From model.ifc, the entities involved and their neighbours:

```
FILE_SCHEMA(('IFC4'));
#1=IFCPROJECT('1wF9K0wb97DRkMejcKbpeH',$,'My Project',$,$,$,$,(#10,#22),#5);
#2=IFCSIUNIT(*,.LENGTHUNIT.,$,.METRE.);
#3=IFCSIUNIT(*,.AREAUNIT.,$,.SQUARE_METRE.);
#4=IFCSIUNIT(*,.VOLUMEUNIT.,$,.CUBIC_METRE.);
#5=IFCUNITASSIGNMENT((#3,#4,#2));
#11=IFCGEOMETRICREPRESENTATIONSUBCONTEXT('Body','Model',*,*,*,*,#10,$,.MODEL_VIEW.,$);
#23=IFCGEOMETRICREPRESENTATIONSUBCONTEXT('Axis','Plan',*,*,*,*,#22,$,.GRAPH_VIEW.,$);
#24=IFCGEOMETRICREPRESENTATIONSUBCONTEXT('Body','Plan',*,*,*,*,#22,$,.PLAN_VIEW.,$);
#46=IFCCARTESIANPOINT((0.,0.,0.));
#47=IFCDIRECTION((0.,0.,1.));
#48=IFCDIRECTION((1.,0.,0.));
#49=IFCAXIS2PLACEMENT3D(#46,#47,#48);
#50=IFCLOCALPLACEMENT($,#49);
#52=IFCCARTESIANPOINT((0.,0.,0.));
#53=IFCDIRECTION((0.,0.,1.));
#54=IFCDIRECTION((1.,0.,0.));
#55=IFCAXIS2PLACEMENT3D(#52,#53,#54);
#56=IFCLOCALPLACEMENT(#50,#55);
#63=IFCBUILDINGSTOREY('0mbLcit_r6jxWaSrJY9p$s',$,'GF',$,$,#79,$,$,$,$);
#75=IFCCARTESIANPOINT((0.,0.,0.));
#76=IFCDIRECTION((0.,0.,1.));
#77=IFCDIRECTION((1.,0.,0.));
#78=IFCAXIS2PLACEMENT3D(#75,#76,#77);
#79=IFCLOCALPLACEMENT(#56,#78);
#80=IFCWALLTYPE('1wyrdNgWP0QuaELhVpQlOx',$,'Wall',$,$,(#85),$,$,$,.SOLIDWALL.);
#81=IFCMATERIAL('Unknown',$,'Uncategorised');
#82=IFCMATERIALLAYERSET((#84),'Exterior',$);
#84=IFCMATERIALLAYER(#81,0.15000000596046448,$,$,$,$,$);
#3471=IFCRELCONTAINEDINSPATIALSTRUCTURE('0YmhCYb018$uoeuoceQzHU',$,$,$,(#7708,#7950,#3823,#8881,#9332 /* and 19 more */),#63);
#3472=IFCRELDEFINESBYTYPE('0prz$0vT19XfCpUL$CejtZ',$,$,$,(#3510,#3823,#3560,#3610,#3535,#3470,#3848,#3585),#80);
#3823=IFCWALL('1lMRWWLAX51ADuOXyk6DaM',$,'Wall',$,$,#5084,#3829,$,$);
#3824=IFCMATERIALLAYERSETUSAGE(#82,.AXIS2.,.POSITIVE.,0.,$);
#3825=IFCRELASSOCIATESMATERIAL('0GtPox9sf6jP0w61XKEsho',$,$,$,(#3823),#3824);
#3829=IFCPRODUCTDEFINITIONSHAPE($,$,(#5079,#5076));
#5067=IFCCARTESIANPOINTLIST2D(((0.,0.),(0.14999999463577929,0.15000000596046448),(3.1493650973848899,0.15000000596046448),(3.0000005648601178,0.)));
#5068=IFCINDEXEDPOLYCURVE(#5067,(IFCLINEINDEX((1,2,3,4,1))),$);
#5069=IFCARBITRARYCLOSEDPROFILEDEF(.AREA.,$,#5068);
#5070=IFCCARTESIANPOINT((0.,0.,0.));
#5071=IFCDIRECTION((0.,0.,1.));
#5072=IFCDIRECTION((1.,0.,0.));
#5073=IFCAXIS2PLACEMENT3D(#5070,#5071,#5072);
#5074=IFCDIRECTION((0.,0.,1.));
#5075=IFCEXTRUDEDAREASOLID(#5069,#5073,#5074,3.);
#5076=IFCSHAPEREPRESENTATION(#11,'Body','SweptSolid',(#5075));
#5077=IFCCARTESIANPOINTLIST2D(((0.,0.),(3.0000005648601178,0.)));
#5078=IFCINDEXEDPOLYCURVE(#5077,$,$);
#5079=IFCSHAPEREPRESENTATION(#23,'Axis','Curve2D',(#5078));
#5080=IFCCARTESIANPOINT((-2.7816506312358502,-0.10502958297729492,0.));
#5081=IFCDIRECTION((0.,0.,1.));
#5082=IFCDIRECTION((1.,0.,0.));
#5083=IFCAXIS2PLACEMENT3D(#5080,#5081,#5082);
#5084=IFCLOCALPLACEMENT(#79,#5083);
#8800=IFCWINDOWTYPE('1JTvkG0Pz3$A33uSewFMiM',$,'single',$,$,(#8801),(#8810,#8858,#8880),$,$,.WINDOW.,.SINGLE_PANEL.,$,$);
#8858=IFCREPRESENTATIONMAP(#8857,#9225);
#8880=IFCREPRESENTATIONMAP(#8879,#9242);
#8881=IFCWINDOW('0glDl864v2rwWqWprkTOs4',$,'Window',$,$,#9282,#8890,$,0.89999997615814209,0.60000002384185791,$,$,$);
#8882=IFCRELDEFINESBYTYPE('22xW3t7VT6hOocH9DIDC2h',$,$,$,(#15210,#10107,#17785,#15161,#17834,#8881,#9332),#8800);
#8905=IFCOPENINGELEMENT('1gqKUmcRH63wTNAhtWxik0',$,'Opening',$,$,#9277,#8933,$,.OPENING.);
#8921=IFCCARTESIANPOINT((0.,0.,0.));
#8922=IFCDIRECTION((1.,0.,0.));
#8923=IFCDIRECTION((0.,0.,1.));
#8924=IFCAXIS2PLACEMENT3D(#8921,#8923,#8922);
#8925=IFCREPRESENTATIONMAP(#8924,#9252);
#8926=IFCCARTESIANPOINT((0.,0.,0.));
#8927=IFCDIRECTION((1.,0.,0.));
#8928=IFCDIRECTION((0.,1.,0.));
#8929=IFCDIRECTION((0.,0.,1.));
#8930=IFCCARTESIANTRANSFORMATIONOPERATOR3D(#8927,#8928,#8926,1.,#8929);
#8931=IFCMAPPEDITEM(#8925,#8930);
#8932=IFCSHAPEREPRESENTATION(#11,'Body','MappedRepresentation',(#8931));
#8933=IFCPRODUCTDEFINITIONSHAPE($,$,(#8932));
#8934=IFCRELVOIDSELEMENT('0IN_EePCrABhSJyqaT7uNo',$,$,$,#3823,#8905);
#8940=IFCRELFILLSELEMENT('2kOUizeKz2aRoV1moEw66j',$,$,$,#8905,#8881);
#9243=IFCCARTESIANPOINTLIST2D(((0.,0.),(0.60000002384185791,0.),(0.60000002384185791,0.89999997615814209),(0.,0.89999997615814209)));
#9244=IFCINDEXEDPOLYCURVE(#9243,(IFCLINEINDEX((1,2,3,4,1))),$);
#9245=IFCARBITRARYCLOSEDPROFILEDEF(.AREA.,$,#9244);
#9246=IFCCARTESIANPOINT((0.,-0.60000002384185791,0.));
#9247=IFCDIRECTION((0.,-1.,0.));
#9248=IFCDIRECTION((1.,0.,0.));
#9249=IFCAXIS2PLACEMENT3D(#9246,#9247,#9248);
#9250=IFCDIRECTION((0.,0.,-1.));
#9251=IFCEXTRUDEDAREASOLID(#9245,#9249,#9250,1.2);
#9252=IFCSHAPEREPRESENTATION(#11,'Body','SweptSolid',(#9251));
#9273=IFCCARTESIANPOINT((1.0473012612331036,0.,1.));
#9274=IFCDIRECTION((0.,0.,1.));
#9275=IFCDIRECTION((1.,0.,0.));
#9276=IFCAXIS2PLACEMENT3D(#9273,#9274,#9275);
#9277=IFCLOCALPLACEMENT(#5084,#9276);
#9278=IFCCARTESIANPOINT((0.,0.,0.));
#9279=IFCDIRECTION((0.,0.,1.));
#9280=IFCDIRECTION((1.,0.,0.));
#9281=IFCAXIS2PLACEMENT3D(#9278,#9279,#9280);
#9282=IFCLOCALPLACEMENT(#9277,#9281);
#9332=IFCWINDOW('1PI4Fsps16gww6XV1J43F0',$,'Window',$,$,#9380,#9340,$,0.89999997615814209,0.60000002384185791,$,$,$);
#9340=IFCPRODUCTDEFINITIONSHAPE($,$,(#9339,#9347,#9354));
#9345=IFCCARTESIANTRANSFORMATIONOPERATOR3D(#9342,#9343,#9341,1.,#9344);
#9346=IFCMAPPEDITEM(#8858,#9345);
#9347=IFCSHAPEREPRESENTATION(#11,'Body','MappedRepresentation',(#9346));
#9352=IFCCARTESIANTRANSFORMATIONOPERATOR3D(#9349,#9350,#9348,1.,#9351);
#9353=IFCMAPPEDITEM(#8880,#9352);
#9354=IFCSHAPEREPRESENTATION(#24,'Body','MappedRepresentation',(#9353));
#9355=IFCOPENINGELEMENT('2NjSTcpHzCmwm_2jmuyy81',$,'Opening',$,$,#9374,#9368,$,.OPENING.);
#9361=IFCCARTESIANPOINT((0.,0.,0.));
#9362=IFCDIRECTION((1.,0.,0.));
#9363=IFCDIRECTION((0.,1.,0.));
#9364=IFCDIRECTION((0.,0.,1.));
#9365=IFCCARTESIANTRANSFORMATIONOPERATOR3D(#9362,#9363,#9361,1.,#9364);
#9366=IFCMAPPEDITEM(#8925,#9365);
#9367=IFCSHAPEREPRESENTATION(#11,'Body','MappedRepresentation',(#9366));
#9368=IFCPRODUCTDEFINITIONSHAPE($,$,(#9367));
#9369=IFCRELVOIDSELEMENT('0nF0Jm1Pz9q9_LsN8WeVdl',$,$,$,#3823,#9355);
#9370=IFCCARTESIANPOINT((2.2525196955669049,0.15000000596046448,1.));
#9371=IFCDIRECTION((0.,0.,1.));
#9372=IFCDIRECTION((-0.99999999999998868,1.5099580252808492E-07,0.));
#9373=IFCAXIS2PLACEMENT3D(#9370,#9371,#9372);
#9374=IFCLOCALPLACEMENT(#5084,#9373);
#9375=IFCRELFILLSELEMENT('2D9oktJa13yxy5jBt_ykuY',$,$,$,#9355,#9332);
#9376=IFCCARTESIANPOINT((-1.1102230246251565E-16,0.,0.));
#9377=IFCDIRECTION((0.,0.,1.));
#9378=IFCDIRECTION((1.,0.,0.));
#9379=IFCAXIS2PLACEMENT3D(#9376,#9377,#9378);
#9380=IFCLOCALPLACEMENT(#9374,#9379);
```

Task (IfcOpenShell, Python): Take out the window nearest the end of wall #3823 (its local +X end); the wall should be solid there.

```python
import ifcopenshell
import ifcopenshell.api.feature
import ifcopenshell.api.root
import ifcopenshell.geom
import ifcopenshell.util.shape

model = ifcopenshell.open("model.ifc")
settings = ifcopenshell.geom.settings()


def volume(element):
    """Net volume in cubic metres, openings subtracted."""
    shape = ifcopenshell.geom.create_shape(settings, element)
    return ifcopenshell.util.shape.get_volume(shape.geometry)


window = model.by_guid("1PI4Fsps16gww6XV1J43F0")
opening = window.FillsVoids[0].RelatingOpeningElement
wall = opening.VoidsElements[0].RelatingBuildingElement
before = volume(wall)

ifcopenshell.api.root.remove_product(model, product=window)
ifcopenshell.api.feature.remove_feature(model, feature=opening)

after = volume(wall)

print(f"wall volume {before:.3f} -> {after:.3f} m3")

model.write("model_rev.ifc")
```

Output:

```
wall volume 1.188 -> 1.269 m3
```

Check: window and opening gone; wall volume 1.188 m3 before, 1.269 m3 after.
